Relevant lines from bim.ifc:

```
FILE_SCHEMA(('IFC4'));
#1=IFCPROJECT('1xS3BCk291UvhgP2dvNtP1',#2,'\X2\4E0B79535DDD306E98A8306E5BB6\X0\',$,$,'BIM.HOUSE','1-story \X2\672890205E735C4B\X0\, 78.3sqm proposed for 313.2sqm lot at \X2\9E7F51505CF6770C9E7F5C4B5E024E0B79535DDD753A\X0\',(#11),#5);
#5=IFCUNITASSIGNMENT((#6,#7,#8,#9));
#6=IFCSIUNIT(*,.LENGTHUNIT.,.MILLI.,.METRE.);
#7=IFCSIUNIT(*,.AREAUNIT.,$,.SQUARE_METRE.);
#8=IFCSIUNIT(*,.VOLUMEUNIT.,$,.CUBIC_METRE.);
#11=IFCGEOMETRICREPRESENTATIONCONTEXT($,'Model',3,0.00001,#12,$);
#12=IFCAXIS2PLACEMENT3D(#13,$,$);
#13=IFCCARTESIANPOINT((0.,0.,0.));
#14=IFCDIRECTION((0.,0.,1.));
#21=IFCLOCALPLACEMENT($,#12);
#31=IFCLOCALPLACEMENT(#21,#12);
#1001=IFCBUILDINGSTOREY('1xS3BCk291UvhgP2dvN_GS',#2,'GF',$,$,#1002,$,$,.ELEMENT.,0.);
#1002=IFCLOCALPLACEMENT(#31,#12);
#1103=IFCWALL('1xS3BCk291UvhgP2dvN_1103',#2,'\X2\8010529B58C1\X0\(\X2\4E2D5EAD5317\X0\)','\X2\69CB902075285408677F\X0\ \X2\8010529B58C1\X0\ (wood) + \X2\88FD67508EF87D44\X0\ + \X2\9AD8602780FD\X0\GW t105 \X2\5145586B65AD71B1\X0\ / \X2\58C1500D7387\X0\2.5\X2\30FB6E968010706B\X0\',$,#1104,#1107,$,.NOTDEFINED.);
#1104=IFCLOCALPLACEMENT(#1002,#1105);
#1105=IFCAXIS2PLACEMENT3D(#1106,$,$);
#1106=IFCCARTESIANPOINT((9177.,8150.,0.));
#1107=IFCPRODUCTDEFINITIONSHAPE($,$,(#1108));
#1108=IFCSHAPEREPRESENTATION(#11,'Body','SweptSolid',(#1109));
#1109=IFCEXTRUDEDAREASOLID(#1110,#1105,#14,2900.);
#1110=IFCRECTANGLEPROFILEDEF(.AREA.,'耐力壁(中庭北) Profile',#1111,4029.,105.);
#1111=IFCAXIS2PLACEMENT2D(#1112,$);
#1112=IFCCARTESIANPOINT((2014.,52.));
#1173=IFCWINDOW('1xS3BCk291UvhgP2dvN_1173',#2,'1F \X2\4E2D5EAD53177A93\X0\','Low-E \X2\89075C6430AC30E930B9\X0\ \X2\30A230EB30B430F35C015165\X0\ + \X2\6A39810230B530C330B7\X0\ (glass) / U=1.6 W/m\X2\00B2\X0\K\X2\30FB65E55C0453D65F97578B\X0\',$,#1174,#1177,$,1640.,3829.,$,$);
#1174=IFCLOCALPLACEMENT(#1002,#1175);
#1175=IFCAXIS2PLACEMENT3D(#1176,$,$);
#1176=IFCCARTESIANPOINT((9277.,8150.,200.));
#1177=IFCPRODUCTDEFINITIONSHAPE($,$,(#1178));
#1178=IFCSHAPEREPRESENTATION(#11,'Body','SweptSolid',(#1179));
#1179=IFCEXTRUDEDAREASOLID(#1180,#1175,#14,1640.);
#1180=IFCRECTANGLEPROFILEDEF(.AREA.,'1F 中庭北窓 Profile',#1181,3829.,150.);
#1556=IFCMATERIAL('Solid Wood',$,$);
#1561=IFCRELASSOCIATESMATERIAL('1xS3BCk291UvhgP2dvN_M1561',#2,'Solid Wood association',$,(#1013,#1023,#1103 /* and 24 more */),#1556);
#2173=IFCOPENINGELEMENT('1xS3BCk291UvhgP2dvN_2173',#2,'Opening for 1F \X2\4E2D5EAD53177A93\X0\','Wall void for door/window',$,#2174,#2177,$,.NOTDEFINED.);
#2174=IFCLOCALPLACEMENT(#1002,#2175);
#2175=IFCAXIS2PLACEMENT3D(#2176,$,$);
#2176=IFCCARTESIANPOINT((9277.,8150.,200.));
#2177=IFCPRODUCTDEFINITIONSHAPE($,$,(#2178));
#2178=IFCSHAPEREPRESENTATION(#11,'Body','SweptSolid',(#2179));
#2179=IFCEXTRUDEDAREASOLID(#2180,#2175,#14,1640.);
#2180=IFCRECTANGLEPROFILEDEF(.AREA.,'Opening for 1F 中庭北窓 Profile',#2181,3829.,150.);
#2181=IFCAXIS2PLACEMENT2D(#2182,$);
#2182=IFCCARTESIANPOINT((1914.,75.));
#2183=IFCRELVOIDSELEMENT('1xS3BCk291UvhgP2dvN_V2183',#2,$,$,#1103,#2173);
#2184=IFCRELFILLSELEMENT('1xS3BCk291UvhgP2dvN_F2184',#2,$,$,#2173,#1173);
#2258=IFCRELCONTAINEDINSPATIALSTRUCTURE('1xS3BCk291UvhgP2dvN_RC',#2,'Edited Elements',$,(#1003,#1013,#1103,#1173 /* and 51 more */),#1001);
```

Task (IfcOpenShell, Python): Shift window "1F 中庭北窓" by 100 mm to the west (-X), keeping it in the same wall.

```python
import ifcopenshell
import ifcopenshell.api.geometry
import ifcopenshell.util.placement
import ifcopenshell.util.unit

model = ifcopenshell.open("bim.ifc")
unit_scale = ifcopenshell.util.unit.calculate_unit_scale(model)

window = model.by_id(1173)
opening = window.FillsVoids[0].RelatingOpeningElement
wall = opening.VoidsElements[0].RelatingBuildingElement

wall_matrix = ifcopenshell.util.placement.get_local_placement(wall.ObjectPlacement)
shift = wall_matrix[:3, 0] * -0.1 / unit_scale
before = ifcopenshell.util.placement.get_local_placement(window.ObjectPlacement)[:3, 3].copy()

# The window is not placed relative to its opening, so move both.
for product in (opening, window):
    matrix = ifcopenshell.util.placement.get_local_placement(product.ObjectPlacement)
    matrix[:3, 3] += shift
    ifcopenshell.api.geometry.edit_object_placement(model, product=product, matrix=matrix, is_si=False)

after = ifcopenshell.util.placement.get_local_placement(window.ObjectPlacement)[:3, 3]
print("window moved by", (after - before).round(3) + 0.0)

model.write("bim_rev.ifc")
```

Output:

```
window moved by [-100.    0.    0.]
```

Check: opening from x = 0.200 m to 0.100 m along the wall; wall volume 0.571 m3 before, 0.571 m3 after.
